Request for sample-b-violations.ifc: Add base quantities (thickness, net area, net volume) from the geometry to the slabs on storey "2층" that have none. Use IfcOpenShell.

First a look at what the model holds.

```python
import ifcopenshell
import ifcopenshell.util.element
import ifcopenshell.util.unit

model = ifcopenshell.open("sample-b-violations.ifc")
print(model.schema)
for unit_type in ("LENGTHUNIT", "AREAUNIT", "VOLUMEUNIT"):
    print(unit_type, ifcopenshell.util.unit.calculate_unit_scale(model, unit_type))
storey = next(s for s in model.by_type("IfcBuildingStorey") if s.Name == "2층")
slabs = [e for e in ifcopenshell.util.element.get_decomposition(storey) if e.is_a("IfcSlab")]
for e in sorted(slabs, key=lambda e: e.id()):
    print(e.id(), e.is_a(), e.Name, list(ifcopenshell.util.element.get_psets(e, qtos_only=True)), sep=" | ")
```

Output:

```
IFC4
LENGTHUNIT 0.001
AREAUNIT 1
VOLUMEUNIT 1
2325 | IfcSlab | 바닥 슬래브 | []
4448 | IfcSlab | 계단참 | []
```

```python
import ifcopenshell
import ifcopenshell.api.pset
import ifcopenshell.geom
import ifcopenshell.util.element
import ifcopenshell.util.shape
import ifcopenshell.util.unit

model = ifcopenshell.open("sample-b-violations.ifc")
unit_scale = ifcopenshell.util.unit.calculate_unit_scale(model)
area_scale = ifcopenshell.util.unit.calculate_unit_scale(model, "AREAUNIT")
volume_scale = ifcopenshell.util.unit.calculate_unit_scale(model, "VOLUMEUNIT")
settings = ifcopenshell.geom.settings()

storey = next(s for s in model.by_type("IfcBuildingStorey") if s.Name == "2층")
slabs = [e for e in ifcopenshell.util.element.get_decomposition(storey) if e.is_a("IfcSlab")]

for e in sorted(slabs, key=lambda e: e.id()):
    if ifcopenshell.util.element.get_psets(e, qtos_only=True, should_inherit=False):
        continue
    # Geometry comes back in metres, in the element's own axes.
    shape = ifcopenshell.geom.create_shape(settings, e)
    values = {
        "Width": ifcopenshell.util.shape.get_z(shape.geometry) / unit_scale,
        "NetArea": ifcopenshell.util.shape.get_footprint_area(shape.geometry) / area_scale,
        "NetVolume": ifcopenshell.util.shape.get_volume(shape.geometry) / volume_scale,
    }
    qto = ifcopenshell.api.pset.add_qto(model, product=e, name="Qto_SlabBaseQuantities")
    ifcopenshell.api.pset.edit_qto(model, qto=qto, properties=values)
    print(e.id(), {k: round(v, 3) for k, v in values.items()})

model.write("sample-b-violations-out.ifc")
```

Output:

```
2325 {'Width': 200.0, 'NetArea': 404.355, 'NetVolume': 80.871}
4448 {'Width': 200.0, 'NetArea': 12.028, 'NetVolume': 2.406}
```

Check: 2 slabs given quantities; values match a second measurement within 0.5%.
